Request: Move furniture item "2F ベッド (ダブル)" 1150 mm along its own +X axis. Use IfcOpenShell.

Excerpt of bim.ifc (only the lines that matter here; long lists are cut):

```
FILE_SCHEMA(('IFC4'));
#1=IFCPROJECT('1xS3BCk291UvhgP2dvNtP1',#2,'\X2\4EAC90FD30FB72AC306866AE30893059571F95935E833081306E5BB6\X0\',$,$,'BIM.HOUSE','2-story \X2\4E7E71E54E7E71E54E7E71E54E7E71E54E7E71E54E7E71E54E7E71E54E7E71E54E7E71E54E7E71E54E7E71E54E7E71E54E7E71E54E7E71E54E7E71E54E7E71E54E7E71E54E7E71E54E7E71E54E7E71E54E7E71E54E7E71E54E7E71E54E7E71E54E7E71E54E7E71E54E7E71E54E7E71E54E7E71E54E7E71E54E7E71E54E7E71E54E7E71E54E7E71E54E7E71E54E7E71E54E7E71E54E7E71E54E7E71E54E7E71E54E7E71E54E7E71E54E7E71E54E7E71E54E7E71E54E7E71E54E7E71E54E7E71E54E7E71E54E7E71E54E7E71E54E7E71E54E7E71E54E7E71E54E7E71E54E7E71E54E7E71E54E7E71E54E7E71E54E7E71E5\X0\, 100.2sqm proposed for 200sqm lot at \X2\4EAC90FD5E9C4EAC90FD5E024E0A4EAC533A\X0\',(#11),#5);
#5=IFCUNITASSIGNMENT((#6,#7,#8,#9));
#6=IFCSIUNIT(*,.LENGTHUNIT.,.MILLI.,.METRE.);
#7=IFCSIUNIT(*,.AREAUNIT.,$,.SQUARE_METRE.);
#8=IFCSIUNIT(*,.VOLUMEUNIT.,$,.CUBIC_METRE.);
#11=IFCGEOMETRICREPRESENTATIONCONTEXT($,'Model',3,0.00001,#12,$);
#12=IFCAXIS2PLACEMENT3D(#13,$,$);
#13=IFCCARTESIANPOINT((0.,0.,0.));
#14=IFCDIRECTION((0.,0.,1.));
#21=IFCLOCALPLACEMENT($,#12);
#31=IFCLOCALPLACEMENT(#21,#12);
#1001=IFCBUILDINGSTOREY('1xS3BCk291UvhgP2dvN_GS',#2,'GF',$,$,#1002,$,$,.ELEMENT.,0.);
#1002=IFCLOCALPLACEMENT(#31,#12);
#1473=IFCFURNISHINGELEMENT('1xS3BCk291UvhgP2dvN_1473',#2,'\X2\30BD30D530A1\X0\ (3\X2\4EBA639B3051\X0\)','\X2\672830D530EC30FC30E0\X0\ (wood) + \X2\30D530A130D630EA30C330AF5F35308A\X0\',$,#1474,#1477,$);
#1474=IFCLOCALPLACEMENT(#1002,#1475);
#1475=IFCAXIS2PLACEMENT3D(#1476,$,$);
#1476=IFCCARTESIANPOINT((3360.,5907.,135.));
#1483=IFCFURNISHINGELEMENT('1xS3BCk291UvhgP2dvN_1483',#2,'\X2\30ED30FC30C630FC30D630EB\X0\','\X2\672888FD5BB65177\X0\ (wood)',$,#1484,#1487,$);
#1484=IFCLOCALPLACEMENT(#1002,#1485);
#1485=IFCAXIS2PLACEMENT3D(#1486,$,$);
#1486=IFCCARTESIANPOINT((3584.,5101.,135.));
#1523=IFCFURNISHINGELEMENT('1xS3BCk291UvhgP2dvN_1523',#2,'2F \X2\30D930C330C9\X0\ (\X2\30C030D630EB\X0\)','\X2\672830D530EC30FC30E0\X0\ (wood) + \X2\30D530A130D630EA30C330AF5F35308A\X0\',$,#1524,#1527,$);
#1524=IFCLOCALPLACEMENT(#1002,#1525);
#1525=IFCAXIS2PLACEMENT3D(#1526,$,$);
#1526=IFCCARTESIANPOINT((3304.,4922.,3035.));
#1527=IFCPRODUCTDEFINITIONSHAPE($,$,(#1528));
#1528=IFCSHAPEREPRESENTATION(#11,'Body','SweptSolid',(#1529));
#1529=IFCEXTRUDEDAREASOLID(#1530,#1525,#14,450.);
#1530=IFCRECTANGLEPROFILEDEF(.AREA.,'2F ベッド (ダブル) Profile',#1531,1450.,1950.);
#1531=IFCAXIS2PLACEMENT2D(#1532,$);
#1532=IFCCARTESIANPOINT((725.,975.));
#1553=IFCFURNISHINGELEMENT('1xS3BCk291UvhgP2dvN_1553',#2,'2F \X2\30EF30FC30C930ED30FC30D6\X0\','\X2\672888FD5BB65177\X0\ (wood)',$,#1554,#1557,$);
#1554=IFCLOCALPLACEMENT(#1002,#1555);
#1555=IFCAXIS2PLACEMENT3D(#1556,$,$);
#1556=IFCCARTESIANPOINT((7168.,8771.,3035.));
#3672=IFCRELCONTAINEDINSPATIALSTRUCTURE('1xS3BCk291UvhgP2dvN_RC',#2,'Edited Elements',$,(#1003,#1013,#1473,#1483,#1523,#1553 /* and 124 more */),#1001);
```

```python
import ifcopenshell
import ifcopenshell.api.geometry
import ifcopenshell.util.placement

model = ifcopenshell.open("bim.ifc")

item = model.by_guid("1xS3BCk291UvhgP2dvN_1523")
matrix = ifcopenshell.util.placement.get_local_placement(item.ObjectPlacement)
matrix[:3, 3] += matrix[:3, 0] * 1150.0
ifcopenshell.api.geometry.edit_object_placement(model, product=item, matrix=matrix, is_si=False)

print(ifcopenshell.util.placement.get_local_placement(item.ObjectPlacement).round(3) + 0.0)

model.write("bim_v2.ifc")
```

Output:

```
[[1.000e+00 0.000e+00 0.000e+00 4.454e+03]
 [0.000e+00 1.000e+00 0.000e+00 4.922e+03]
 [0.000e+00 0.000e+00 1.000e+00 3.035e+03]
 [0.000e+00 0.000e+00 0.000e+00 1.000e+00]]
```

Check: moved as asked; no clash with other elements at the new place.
